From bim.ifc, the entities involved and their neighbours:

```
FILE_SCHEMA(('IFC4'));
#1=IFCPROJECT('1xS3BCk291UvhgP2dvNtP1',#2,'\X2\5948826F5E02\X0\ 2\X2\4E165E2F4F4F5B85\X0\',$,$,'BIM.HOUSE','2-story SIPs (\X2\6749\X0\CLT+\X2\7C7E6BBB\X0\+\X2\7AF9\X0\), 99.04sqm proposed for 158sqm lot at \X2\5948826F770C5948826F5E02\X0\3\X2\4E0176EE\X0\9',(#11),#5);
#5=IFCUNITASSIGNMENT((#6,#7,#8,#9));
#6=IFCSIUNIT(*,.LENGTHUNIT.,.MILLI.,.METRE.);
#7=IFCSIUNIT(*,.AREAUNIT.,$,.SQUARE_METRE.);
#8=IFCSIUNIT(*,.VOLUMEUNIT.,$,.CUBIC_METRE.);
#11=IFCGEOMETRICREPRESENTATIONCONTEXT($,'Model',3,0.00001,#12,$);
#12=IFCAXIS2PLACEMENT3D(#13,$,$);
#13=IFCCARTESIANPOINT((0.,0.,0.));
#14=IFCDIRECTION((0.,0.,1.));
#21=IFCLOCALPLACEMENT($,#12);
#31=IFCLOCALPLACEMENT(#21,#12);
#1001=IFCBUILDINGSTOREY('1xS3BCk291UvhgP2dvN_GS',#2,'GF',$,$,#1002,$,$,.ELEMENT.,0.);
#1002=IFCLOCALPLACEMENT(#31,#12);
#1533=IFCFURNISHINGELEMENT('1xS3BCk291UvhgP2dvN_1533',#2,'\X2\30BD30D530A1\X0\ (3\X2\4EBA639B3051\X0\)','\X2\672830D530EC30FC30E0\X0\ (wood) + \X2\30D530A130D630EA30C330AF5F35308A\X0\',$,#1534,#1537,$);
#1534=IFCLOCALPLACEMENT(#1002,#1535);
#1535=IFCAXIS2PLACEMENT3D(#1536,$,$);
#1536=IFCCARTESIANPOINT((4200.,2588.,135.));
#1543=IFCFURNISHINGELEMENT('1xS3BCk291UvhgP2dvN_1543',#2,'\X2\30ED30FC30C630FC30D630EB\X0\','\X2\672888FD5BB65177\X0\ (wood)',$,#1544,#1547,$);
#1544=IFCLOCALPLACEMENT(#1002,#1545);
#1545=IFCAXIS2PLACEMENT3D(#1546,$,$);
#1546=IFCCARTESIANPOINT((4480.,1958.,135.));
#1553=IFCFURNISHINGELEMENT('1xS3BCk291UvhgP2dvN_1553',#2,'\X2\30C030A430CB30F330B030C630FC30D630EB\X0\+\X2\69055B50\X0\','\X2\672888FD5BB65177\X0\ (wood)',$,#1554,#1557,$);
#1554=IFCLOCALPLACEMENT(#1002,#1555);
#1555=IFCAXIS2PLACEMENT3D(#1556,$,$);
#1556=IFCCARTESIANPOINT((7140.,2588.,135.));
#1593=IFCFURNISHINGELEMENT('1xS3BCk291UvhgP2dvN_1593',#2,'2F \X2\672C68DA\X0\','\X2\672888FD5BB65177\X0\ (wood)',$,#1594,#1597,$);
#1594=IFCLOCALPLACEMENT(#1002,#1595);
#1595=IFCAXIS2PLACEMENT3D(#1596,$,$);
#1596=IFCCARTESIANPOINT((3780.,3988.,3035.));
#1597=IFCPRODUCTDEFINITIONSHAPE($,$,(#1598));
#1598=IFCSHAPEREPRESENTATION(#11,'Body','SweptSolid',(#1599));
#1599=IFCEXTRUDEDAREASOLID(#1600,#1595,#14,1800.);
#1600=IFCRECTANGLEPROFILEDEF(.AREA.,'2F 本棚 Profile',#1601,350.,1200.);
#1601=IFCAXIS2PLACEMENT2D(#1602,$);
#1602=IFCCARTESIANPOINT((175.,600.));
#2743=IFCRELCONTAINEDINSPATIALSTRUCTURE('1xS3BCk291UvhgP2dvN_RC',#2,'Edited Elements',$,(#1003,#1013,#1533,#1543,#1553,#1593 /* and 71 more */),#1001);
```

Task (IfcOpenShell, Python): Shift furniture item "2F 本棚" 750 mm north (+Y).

```python
import ifcopenshell
import ifcopenshell.api.geometry
import ifcopenshell.util.placement
import ifcopenshell.util.unit

model = ifcopenshell.open("bim.ifc")
unit_scale = ifcopenshell.util.unit.calculate_unit_scale(model)

item = model.by_id(1593)
matrix = ifcopenshell.util.placement.get_local_placement(item.ObjectPlacement)
matrix[1, 3] += 0.75 / unit_scale
ifcopenshell.api.geometry.edit_object_placement(model, product=item, matrix=matrix, is_si=False)

print(ifcopenshell.util.placement.get_local_placement(item.ObjectPlacement).round(3) + 0.0)

model.write("bim_v2.ifc")
```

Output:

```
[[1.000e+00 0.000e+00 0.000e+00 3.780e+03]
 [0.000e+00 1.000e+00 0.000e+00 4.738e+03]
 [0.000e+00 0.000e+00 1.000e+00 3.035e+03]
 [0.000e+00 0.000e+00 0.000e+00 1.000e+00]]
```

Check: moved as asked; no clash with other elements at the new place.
